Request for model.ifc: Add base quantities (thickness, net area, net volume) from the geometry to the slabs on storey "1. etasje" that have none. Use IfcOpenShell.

First a look at what the model holds.

```python
import ifcopenshell
import ifcopenshell.util.element
import ifcopenshell.util.unit

model = ifcopenshell.open("model.ifc")
print(model.schema)
for unit_type in ("LENGTHUNIT", "AREAUNIT", "VOLUMEUNIT"):
    print(unit_type, ifcopenshell.util.unit.calculate_unit_scale(model, unit_type))
storey = next(s for s in model.by_type("IfcBuildingStorey") if s.Name == "1. etasje")
slabs = [e for e in ifcopenshell.util.element.get_decomposition(storey) if e.is_a("IfcSlab")]
for e in sorted(slabs, key=lambda e: e.id()):
    print(e.id(), e.is_a(), e.Name, list(ifcopenshell.util.element.get_psets(e, qtos_only=True)), sep=" | ")
```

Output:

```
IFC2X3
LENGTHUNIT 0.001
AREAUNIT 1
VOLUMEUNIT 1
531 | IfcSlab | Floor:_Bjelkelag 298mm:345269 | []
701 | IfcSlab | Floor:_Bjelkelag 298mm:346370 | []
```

```python
import ifcopenshell
import ifcopenshell.api.pset
import ifcopenshell.geom
import ifcopenshell.util.element
import ifcopenshell.util.shape
import ifcopenshell.util.unit

model = ifcopenshell.open("model.ifc")
unit_scale = ifcopenshell.util.unit.calculate_unit_scale(model)
area_scale = ifcopenshell.util.unit.calculate_unit_scale(model, "AREAUNIT")
volume_scale = ifcopenshell.util.unit.calculate_unit_scale(model, "VOLUMEUNIT")
settings = ifcopenshell.geom.settings()

storey = next(s for s in model.by_type("IfcBuildingStorey") if s.Name == "1. etasje")
slabs = [e for e in ifcopenshell.util.element.get_decomposition(storey) if e.is_a("IfcSlab")]

for e in sorted(slabs, key=lambda e: e.id()):
    if ifcopenshell.util.element.get_psets(e, qtos_only=True, should_inherit=False):
        continue
    # Geometry comes back in metres, in the element's own axes.
    shape = ifcopenshell.geom.create_shape(settings, e)
    values = {
        "Width": ifcopenshell.util.shape.get_z(shape.geometry) / unit_scale,
        "NetArea": ifcopenshell.util.shape.get_footprint_area(shape.geometry) / area_scale,
        "NetVolume": ifcopenshell.util.shape.get_volume(shape.geometry) / volume_scale,
    }
    qto = ifcopenshell.api.pset.add_qto(model, product=e, name="BaseQuantities")
    ifcopenshell.api.pset.edit_qto(model, qto=qto, properties=values)
    print(e.id(), {k: round(v, 3) for k, v in values.items()})

model.write("model-out.ifc")
```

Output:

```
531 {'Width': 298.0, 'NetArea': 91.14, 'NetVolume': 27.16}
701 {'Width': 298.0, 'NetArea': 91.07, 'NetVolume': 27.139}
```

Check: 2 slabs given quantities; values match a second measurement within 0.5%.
